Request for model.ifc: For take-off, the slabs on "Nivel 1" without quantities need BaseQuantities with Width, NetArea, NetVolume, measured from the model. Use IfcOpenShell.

First a look at what the model holds.

```python
import ifcopenshell
import ifcopenshell.util.element
import ifcopenshell.util.unit

model = ifcopenshell.open("model.ifc")
print(model.schema)
for unit_type in ("LENGTHUNIT", "AREAUNIT", "VOLUMEUNIT"):
    print(unit_type, ifcopenshell.util.unit.calculate_unit_scale(model, unit_type))
storey = next(s for s in model.by_type("IfcBuildingStorey") if s.Name == "Nivel 1")
slabs = [e for e in ifcopenshell.util.element.get_decomposition(storey) if e.is_a("IfcSlab")]
for e in sorted(slabs, key=lambda e: e.id()):
    print(e.id(), e.is_a(), e.Name, list(ifcopenshell.util.element.get_psets(e, qtos_only=True)), sep=" | ")
```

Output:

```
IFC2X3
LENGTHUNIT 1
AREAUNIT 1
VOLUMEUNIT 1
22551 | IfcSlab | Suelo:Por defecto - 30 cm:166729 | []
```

```python
import ifcopenshell
import ifcopenshell.api.pset
import ifcopenshell.geom
import ifcopenshell.util.element
import ifcopenshell.util.shape
import ifcopenshell.util.unit

model = ifcopenshell.open("model.ifc")
unit_scale = ifcopenshell.util.unit.calculate_unit_scale(model)
area_scale = ifcopenshell.util.unit.calculate_unit_scale(model, "AREAUNIT")
volume_scale = ifcopenshell.util.unit.calculate_unit_scale(model, "VOLUMEUNIT")
settings = ifcopenshell.geom.settings()

storey = next(s for s in model.by_type("IfcBuildingStorey") if s.Name == "Nivel 1")
slabs = [e for e in ifcopenshell.util.element.get_decomposition(storey) if e.is_a("IfcSlab")]

for e in sorted(slabs, key=lambda e: e.id()):
    if ifcopenshell.util.element.get_psets(e, qtos_only=True, should_inherit=False):
        continue
    # Geometry comes back in metres, in the element's own axes.
    shape = ifcopenshell.geom.create_shape(settings, e)
    values = {
        "Width": ifcopenshell.util.shape.get_z(shape.geometry) / unit_scale,
        "NetArea": ifcopenshell.util.shape.get_footprint_area(shape.geometry) / area_scale,
        "NetVolume": ifcopenshell.util.shape.get_volume(shape.geometry) / volume_scale,
    }
    qto = ifcopenshell.api.pset.add_qto(model, product=e, name="BaseQuantities")
    ifcopenshell.api.pset.edit_qto(model, qto=qto, properties=values)
    print(e.id(), {k: round(v, 3) for k, v in values.items()})

model.write("model_v2.ifc")
```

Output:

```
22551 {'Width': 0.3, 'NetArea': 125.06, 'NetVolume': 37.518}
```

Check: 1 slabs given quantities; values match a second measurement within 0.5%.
